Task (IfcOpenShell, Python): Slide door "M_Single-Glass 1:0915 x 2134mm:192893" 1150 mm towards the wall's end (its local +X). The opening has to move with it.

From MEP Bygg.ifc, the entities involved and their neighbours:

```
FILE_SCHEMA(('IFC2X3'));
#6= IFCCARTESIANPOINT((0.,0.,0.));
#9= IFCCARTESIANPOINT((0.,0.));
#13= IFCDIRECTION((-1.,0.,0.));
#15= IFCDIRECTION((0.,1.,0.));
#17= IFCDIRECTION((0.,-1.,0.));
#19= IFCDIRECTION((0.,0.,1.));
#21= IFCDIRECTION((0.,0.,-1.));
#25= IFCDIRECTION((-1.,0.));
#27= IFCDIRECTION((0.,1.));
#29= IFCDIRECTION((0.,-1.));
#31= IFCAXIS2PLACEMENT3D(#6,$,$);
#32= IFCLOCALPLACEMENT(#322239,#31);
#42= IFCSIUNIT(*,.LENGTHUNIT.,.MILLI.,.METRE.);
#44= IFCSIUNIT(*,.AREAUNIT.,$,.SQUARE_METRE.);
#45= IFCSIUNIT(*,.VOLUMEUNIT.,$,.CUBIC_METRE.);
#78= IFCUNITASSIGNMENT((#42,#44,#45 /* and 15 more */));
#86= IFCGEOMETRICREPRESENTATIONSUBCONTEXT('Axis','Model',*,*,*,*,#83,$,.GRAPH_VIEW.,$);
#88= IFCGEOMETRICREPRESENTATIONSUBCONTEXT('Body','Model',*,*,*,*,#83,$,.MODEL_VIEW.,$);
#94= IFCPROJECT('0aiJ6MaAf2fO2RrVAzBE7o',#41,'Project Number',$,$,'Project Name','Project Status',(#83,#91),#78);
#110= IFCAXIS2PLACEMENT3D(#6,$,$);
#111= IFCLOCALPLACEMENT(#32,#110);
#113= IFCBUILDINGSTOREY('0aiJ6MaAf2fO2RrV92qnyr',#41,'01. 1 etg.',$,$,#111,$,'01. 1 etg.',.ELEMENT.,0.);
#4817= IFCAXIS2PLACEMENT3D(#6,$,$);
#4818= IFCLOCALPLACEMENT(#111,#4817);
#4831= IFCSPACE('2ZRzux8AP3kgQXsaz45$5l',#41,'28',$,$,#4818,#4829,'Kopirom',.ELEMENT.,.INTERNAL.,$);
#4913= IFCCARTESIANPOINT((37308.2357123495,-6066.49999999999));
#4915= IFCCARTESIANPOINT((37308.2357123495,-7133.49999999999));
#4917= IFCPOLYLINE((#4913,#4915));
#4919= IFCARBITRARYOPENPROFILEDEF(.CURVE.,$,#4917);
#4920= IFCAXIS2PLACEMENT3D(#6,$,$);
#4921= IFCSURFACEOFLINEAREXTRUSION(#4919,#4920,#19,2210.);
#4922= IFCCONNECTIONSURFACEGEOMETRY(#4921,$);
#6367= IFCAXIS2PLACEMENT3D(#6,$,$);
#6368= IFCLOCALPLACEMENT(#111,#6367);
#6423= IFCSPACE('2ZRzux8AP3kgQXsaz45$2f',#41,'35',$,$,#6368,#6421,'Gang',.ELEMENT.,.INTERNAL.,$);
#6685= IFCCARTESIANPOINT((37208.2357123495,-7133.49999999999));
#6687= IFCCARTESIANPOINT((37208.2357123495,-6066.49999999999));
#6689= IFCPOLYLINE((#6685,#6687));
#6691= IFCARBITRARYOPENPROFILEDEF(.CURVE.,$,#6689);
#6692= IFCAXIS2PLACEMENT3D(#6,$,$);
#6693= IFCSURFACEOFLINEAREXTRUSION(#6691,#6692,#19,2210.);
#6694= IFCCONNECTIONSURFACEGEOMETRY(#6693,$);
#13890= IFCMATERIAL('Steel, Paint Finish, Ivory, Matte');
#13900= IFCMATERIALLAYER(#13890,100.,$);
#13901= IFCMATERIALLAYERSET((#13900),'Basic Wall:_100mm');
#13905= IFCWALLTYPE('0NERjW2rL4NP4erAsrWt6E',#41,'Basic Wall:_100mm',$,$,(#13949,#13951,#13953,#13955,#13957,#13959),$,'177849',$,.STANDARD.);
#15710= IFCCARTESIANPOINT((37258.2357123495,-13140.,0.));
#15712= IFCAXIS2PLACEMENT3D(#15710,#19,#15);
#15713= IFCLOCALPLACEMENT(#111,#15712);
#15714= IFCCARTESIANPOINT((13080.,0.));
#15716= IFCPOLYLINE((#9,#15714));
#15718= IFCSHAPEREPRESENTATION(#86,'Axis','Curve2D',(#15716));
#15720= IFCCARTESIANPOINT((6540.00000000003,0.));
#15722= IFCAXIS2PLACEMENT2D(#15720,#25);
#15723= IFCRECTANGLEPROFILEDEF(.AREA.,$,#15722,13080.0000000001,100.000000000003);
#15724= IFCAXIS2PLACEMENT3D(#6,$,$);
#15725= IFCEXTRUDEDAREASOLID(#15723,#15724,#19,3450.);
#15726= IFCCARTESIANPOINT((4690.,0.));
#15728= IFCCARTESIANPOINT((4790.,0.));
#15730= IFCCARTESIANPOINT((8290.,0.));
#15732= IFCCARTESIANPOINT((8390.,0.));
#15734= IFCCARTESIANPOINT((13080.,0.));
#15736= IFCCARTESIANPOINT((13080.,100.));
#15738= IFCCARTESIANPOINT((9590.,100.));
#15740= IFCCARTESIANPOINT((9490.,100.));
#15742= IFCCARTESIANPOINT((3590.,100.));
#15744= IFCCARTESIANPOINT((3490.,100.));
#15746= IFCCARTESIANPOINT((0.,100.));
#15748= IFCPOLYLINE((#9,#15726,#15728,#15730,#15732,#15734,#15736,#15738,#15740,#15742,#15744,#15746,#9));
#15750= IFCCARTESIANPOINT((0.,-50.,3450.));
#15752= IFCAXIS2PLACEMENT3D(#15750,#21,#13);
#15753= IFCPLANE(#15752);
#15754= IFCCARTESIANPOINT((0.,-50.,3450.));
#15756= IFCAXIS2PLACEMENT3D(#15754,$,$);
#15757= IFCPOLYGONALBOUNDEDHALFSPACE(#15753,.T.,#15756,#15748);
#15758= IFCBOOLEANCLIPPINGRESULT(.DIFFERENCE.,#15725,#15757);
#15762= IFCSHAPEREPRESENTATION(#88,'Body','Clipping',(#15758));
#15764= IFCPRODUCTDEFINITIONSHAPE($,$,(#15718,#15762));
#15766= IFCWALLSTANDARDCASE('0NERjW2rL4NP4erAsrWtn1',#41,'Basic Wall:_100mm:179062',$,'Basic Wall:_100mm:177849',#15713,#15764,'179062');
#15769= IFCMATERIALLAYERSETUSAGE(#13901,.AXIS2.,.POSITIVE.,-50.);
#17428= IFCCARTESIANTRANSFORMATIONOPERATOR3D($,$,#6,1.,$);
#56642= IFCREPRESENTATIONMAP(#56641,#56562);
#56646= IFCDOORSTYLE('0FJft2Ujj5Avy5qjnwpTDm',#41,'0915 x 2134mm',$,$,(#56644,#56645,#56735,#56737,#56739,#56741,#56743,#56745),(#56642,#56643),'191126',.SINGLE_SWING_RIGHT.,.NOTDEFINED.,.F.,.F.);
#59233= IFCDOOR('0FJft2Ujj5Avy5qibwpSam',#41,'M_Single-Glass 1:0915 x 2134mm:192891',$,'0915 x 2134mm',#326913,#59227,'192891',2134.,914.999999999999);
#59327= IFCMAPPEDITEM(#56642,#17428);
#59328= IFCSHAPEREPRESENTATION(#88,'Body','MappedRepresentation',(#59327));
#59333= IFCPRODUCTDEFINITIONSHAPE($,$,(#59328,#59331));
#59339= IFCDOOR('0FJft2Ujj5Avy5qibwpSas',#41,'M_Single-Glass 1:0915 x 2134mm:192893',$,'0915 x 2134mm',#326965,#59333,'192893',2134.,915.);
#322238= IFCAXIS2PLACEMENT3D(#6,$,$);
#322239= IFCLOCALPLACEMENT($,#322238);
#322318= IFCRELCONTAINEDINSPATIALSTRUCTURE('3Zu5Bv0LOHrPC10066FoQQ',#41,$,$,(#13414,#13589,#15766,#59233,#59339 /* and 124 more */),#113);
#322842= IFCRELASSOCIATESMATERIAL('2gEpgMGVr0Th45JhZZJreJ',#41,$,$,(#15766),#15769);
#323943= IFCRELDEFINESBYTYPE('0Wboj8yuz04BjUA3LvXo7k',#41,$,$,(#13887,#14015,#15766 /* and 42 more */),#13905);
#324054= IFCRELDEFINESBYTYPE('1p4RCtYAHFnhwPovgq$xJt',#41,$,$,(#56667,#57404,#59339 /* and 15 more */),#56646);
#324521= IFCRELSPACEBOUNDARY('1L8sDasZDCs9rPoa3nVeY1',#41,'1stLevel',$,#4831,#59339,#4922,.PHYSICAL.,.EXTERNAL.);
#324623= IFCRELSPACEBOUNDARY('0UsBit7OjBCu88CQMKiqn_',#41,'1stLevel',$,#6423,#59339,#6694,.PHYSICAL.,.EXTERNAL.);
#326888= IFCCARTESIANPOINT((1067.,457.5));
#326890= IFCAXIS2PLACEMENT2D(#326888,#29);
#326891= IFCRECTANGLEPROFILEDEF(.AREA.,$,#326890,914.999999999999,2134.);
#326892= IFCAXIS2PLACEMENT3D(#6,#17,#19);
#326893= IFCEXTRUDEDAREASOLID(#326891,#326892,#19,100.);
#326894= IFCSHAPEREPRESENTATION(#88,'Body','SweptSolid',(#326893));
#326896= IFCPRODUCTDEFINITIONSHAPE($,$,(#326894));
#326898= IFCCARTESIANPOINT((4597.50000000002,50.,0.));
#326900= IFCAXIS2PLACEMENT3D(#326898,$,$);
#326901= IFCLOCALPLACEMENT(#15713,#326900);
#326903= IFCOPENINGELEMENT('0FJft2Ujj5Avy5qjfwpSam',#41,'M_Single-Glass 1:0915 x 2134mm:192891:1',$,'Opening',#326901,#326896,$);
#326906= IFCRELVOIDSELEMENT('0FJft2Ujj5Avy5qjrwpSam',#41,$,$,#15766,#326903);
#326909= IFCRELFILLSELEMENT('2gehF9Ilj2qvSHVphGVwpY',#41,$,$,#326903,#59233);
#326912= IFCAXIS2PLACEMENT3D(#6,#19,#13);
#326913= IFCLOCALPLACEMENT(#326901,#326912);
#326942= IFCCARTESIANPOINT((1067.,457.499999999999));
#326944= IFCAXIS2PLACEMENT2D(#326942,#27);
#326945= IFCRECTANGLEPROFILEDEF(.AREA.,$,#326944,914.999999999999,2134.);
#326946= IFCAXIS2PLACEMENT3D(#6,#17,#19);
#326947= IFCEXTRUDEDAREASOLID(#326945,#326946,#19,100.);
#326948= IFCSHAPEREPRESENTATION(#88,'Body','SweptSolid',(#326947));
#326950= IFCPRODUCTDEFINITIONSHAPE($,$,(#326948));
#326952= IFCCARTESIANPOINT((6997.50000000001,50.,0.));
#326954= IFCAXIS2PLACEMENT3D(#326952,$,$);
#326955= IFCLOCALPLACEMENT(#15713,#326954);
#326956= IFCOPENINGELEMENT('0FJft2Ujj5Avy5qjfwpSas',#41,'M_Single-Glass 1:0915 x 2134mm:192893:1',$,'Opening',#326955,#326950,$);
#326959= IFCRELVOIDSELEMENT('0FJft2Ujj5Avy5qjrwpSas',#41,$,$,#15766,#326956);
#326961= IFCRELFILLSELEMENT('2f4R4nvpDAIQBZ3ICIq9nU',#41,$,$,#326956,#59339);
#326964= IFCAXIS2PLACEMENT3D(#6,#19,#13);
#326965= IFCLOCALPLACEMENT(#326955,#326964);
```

```python
import numpy as np
import ifcopenshell
import ifcopenshell.api.geometry
import ifcopenshell.util.placement
import ifcopenshell.util.unit

model = ifcopenshell.open("MEP Bygg.ifc")
unit_scale = ifcopenshell.util.unit.calculate_unit_scale(model)

door = model.by_guid("0FJft2Ujj5Avy5qibwpSas")
opening = door.FillsVoids[0].RelatingOpeningElement
wall = opening.VoidsElements[0].RelatingBuildingElement

wall_matrix = ifcopenshell.util.placement.get_local_placement(wall.ObjectPlacement)
shift = wall_matrix[:3, 0] * 1.15 / unit_scale
before = ifcopenshell.util.placement.get_local_placement(door.ObjectPlacement)[:3, 3].copy()

# The door is placed relative to its opening, so it follows when the opening moves.
matrix = ifcopenshell.util.placement.get_local_placement(opening.ObjectPlacement)
matrix[:3, 3] += shift
ifcopenshell.api.geometry.edit_object_placement(
    model, product=opening, matrix=matrix, is_si=False, should_transform_children=True
)

# Space boundary surfaces are stored in each space's coordinates; move them too.
for rel in door.ProvidesBoundaries:
    if not rel.ConnectionGeometry:
        continue
    surface = rel.ConnectionGeometry.SurfaceOnRelatingElement
    space_matrix = ifcopenshell.util.placement.get_local_placement(rel.RelatingSpace.ObjectPlacement)
    point = np.array(surface.Position.Location.Coordinates) + space_matrix[:3, :3].T @ shift
    surface.Position = model.createIfcAxis2Placement3D(
        model.createIfcCartesianPoint(point.tolist()), surface.Position.Axis, surface.Position.RefDirection
    )

after = ifcopenshell.util.placement.get_local_placement(door.ObjectPlacement)[:3, 3]
print("door moved by", (after - before).round(3) + 0.0)

model.write("MEP Bygg-out.ifc")
```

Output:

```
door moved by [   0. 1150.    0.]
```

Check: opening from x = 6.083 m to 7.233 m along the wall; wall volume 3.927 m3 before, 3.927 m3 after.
